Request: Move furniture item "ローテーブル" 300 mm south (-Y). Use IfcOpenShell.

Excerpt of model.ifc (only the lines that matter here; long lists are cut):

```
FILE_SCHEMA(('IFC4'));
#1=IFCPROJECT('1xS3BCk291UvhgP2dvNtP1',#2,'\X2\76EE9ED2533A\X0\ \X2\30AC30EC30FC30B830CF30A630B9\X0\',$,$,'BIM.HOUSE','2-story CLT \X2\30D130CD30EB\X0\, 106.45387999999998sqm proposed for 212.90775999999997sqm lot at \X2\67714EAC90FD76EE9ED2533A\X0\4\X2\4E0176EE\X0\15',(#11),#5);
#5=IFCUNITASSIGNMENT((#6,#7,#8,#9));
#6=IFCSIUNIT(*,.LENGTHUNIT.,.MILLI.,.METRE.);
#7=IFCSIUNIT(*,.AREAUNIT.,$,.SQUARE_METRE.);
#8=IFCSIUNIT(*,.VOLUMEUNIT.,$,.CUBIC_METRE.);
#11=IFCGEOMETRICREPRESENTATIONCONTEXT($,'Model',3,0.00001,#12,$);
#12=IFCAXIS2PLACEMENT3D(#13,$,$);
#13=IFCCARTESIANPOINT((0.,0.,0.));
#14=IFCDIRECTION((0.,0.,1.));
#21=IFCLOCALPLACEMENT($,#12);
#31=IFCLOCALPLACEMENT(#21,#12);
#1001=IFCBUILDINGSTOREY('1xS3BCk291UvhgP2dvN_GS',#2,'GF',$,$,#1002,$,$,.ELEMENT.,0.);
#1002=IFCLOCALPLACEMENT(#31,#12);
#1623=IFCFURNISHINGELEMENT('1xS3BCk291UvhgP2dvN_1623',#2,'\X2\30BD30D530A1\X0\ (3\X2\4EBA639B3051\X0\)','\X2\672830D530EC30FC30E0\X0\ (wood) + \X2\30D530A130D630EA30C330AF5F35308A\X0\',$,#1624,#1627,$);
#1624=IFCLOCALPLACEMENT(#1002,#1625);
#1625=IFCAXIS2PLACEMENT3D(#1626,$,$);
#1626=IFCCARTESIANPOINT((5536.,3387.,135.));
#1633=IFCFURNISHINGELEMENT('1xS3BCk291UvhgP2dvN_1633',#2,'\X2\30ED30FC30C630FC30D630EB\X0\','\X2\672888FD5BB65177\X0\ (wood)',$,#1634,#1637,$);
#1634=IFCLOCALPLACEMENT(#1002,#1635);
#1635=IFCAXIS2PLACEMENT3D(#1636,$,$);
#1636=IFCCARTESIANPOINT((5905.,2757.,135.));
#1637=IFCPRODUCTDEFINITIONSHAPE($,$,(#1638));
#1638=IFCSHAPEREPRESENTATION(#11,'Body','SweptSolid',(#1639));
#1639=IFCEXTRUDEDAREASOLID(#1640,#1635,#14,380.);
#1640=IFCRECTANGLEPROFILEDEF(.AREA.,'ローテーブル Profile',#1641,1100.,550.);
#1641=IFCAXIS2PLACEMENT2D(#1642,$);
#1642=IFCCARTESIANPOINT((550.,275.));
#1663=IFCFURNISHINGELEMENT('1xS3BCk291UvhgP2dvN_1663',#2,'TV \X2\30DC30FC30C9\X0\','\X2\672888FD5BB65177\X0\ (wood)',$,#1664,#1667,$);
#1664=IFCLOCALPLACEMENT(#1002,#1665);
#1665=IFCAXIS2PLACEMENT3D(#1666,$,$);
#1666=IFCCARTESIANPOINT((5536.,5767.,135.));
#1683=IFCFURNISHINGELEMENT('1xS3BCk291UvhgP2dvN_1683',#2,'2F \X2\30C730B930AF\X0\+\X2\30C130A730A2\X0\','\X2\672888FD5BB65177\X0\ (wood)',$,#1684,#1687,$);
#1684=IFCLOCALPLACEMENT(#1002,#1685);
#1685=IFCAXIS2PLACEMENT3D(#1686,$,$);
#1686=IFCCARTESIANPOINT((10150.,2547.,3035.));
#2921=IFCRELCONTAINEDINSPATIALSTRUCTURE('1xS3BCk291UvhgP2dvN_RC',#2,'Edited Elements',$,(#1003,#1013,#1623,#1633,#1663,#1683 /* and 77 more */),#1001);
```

```python
import ifcopenshell
import ifcopenshell.api.geometry
import ifcopenshell.util.placement
import ifcopenshell.util.unit

model = ifcopenshell.open("model.ifc")
unit_scale = ifcopenshell.util.unit.calculate_unit_scale(model)

item = model.by_guid("1xS3BCk291UvhgP2dvN_1633")
matrix = ifcopenshell.util.placement.get_local_placement(item.ObjectPlacement)
matrix[1, 3] -= 0.3 / unit_scale
ifcopenshell.api.geometry.edit_object_placement(model, product=item, matrix=matrix, is_si=False)

print(ifcopenshell.util.placement.get_local_placement(item.ObjectPlacement).round(3) + 0.0)

model.write("model_v2.ifc")
```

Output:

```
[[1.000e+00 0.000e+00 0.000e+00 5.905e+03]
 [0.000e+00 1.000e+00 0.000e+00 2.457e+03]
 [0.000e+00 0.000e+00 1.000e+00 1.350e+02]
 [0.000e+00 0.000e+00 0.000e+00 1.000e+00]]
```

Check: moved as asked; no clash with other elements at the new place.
